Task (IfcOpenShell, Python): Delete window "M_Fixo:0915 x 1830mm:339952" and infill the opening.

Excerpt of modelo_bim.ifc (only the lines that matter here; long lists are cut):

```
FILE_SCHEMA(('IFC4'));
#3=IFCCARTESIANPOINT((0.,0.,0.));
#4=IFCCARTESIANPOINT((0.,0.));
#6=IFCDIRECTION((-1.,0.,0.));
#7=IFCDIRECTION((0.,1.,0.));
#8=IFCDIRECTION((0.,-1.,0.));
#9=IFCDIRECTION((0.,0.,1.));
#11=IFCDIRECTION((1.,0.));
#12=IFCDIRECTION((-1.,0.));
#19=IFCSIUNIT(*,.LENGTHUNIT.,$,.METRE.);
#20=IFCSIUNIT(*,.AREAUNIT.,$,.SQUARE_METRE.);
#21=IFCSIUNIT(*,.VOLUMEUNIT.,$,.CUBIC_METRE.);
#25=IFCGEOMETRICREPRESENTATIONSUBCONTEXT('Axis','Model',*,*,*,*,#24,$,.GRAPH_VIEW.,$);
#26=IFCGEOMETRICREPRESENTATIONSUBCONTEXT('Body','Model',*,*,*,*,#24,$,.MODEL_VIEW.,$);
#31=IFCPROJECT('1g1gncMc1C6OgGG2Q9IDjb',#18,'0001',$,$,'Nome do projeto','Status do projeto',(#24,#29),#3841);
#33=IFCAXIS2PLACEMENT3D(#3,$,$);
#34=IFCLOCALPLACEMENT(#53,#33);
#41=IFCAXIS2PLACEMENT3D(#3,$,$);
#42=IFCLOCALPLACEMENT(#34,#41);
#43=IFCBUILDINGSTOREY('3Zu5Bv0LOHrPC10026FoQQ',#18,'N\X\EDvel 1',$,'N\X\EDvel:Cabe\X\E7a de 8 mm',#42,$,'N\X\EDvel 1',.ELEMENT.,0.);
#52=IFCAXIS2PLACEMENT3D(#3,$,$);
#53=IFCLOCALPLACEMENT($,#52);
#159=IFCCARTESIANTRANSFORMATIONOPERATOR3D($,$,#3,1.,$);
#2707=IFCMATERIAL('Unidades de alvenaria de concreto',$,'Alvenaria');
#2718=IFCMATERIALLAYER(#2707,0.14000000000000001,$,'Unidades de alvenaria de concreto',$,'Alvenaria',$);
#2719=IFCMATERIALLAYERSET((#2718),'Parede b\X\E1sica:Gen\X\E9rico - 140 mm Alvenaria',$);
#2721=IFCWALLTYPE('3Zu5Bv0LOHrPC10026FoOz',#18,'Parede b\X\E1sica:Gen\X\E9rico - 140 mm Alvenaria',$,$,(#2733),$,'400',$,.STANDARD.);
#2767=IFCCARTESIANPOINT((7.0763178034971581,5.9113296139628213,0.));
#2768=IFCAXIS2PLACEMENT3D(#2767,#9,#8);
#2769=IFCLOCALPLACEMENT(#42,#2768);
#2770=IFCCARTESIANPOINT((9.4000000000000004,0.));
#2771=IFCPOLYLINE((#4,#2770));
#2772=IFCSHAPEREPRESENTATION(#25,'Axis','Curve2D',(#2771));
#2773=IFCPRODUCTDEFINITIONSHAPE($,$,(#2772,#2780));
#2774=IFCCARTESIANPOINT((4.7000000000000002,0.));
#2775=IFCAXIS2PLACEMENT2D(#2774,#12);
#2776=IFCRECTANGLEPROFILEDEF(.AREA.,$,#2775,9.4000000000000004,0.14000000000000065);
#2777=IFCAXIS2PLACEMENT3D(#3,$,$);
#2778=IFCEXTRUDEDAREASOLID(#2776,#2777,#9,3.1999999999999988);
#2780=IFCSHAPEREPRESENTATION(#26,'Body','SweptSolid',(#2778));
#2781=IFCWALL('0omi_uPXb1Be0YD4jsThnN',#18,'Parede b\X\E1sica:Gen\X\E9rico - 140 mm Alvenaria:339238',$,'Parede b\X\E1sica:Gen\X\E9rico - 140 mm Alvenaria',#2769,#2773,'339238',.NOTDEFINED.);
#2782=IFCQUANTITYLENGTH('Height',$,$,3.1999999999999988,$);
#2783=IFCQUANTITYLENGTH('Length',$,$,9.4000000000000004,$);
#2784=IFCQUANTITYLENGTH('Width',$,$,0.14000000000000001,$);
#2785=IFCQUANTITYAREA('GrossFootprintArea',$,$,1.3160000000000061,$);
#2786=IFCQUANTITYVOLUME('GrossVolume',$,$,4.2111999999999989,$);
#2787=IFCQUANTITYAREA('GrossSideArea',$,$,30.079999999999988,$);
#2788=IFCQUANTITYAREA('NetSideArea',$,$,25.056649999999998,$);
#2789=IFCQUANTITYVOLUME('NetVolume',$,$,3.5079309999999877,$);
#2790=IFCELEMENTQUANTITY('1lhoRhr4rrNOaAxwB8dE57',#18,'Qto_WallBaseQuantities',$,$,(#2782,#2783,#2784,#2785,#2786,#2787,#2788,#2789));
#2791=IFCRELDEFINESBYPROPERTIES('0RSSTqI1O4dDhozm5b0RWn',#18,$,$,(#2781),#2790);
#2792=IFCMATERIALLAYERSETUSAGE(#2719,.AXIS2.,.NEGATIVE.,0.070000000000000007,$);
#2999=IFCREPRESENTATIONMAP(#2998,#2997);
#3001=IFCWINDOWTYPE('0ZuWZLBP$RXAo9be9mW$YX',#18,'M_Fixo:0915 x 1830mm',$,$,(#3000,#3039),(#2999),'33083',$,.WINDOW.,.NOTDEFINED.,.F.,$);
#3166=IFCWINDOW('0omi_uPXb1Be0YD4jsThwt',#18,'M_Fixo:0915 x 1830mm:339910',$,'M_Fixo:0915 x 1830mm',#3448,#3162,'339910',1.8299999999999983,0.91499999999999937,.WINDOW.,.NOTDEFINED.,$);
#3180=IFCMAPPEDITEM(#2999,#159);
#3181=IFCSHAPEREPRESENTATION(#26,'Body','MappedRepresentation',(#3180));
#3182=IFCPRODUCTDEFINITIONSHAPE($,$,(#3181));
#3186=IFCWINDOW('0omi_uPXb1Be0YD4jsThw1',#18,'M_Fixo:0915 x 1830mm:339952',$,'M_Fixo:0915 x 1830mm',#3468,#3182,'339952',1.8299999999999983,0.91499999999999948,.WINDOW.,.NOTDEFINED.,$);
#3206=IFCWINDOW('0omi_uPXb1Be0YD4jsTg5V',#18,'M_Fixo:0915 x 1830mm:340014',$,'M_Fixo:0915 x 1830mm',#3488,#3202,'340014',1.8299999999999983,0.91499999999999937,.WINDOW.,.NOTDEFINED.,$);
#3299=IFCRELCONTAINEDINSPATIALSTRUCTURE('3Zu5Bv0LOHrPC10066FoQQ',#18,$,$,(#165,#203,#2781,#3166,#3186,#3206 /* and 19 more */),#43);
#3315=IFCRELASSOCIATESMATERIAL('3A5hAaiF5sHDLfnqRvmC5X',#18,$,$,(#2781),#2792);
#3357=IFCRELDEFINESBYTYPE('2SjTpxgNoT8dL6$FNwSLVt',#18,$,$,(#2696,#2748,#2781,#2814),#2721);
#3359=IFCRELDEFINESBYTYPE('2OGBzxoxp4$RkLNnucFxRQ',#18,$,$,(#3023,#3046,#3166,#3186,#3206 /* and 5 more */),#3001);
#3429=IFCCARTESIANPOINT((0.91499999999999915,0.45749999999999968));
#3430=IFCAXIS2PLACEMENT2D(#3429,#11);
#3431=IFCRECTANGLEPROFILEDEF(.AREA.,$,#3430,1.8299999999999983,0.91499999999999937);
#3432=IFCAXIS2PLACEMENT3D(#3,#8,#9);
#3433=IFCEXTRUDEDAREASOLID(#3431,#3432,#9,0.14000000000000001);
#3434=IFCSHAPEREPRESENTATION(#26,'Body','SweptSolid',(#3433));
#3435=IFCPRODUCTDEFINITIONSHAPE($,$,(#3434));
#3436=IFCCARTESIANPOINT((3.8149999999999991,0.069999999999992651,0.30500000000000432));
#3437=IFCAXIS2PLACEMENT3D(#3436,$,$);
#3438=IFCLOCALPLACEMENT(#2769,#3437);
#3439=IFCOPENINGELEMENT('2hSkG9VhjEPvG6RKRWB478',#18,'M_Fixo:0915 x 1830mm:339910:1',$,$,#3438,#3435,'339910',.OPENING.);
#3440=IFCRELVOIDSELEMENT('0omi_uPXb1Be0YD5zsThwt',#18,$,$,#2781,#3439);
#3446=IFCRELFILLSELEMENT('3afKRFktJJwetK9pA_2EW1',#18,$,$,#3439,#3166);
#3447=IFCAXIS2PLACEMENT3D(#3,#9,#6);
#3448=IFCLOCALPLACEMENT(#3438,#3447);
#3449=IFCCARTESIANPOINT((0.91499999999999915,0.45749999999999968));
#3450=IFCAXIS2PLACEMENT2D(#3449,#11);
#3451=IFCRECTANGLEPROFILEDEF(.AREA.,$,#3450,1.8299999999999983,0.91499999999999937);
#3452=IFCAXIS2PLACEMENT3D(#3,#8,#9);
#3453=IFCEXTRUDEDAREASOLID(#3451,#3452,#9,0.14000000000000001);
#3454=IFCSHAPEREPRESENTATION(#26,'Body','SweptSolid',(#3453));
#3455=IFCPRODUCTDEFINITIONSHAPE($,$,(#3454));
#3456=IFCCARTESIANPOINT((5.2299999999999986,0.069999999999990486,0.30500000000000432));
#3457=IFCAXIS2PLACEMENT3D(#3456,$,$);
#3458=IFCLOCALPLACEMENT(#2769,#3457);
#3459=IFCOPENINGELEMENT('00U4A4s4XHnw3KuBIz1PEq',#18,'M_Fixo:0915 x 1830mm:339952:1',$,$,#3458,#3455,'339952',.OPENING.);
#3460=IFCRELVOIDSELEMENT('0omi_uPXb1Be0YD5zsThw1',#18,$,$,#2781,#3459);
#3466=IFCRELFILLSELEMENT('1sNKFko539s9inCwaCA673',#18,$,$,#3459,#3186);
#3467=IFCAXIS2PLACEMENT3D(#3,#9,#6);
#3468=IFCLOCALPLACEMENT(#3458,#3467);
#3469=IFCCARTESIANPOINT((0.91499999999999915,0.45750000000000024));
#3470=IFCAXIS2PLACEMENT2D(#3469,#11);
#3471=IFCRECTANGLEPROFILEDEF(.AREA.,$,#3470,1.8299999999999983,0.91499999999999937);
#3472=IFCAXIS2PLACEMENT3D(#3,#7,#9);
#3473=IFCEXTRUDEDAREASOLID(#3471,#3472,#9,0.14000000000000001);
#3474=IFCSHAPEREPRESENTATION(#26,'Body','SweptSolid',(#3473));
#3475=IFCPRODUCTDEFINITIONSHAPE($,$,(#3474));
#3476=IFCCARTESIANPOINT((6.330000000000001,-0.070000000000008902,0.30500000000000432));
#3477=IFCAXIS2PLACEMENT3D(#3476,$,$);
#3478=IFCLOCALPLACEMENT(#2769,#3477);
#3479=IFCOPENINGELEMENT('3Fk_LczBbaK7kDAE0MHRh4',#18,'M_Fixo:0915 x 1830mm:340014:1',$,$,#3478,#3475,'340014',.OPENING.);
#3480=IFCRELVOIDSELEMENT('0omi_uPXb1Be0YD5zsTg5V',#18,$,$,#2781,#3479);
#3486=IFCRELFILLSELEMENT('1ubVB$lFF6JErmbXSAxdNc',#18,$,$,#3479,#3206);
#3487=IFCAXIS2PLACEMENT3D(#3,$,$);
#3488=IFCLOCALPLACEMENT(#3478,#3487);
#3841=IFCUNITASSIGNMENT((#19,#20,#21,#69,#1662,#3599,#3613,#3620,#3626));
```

```python
import ifcopenshell
import ifcopenshell.api.feature
import ifcopenshell.api.pset
import ifcopenshell.api.root
import ifcopenshell.geom
import ifcopenshell.util.element
import ifcopenshell.util.shape
import ifcopenshell.util.unit

model = ifcopenshell.open("modelo_bim.ifc")
area_scale = ifcopenshell.util.unit.calculate_unit_scale(model, "AREAUNIT")
volume_scale = ifcopenshell.util.unit.calculate_unit_scale(model, "VOLUMEUNIT")
settings = ifcopenshell.geom.settings()


def volume(element):
    """Net volume in cubic metres, openings subtracted."""
    shape = ifcopenshell.geom.create_shape(settings, element)
    return ifcopenshell.util.shape.get_volume(shape.geometry)


window = model.by_id(3186)
opening = window.FillsVoids[0].RelatingOpeningElement
wall = opening.VoidsElements[0].RelatingBuildingElement
before = volume(wall)

ifcopenshell.api.root.remove_product(model, product=window)
ifcopenshell.api.feature.remove_feature(model, feature=opening)

after = volume(wall)
thickness = 0.14  # wall thickness in metres

# Update the wall's stored quantities.
qto = model.by_id(ifcopenshell.util.element.get_pset(wall, "Qto_WallBaseQuantities", should_inherit=False)["id"])
ifcopenshell.api.pset.edit_qto(model, qto=qto, properties={
    "NetSideArea": after / thickness / area_scale,
    "NetVolume": after / volume_scale,
})

print(f"wall volume {before:.3f} -> {after:.3f} m3")

model.write("modelo_bim_v2.ifc")
```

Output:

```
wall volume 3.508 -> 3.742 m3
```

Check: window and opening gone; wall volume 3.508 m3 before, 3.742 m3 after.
